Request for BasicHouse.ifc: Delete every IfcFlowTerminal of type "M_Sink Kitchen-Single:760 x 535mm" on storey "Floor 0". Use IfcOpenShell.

First a look at what the model holds.

```python
import ifcopenshell
import ifcopenshell.util.element

model = ifcopenshell.open("BasicHouse.ifc")
print(model.schema)
storey = next(s for s in model.by_type("IfcBuildingStorey") if s.Name == "Floor 0")
terminals = [e for e in ifcopenshell.util.element.get_decomposition(storey) if e.is_a("IfcFlowTerminal")]
seen = {}
for e in terminals:
    element_type = ifcopenshell.util.element.get_type(e)
    name = element_type.Name if element_type not in (None, e) else None
    seen[name] = seen.get(name, 0) + 1
for name, count in sorted(seen.items(), key=str):
    print(count, "x", name)
```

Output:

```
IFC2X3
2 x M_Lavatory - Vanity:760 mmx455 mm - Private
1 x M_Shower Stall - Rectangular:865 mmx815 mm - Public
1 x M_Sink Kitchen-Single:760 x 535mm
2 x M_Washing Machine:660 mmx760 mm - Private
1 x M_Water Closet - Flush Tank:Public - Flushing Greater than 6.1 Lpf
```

```python
import ifcopenshell
import ifcopenshell.api.root
import ifcopenshell.util.element

model = ifcopenshell.open("BasicHouse.ifc")

storey = next(s for s in model.by_type("IfcBuildingStorey") if s.Name == "Floor 0")
terminals = [e for e in ifcopenshell.util.element.get_decomposition(storey) if e.is_a("IfcFlowTerminal")]
targets = [e for e in terminals if (t := ifcopenshell.util.element.get_type(e)) not in (None, e) and t.Name == "M_Sink Kitchen-Single:760 x 535mm"]

for e in targets:
    ifcopenshell.api.root.remove_product(model, product=e)
print(len(targets), "removed")

model.write("BasicHouse_updated.ifc")
```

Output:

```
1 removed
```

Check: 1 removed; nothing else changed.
